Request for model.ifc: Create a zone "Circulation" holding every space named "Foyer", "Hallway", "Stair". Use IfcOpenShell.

First a look at what the model holds.

```python
import ifcopenshell

model = ifcopenshell.open("model.ifc")
print(model.schema)
seen = {}
for space in model.by_type("IfcSpace"):
    seen[space.LongName] = seen.get(space.LongName, 0) + 1
for name, count in sorted(seen.items(), key=str):
    print(count, "x", name)
print("zones:", [z.Name for z in model.by_type("IfcZone")][:20])
```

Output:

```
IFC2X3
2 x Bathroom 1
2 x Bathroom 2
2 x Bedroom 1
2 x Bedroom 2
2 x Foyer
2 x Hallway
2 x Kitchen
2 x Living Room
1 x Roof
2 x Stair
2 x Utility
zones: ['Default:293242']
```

```python
import ifcopenshell
import ifcopenshell.api.group
import ifcopenshell.api.root

model = ifcopenshell.open("model.ifc")

names = {"Foyer", "Hallway", "Stair"}
spaces = [s for s in model.by_type("IfcSpace") if s.LongName in names]

zone = ifcopenshell.api.root.create_entity(model, ifc_class="IfcZone", name="Circulation")
ifcopenshell.api.group.assign_group(model, products=spaces, group=zone)
print(len(spaces), "spaces in", zone.Name)

model.write("model_updated.ifc")
```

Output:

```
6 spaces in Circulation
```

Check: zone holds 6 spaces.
